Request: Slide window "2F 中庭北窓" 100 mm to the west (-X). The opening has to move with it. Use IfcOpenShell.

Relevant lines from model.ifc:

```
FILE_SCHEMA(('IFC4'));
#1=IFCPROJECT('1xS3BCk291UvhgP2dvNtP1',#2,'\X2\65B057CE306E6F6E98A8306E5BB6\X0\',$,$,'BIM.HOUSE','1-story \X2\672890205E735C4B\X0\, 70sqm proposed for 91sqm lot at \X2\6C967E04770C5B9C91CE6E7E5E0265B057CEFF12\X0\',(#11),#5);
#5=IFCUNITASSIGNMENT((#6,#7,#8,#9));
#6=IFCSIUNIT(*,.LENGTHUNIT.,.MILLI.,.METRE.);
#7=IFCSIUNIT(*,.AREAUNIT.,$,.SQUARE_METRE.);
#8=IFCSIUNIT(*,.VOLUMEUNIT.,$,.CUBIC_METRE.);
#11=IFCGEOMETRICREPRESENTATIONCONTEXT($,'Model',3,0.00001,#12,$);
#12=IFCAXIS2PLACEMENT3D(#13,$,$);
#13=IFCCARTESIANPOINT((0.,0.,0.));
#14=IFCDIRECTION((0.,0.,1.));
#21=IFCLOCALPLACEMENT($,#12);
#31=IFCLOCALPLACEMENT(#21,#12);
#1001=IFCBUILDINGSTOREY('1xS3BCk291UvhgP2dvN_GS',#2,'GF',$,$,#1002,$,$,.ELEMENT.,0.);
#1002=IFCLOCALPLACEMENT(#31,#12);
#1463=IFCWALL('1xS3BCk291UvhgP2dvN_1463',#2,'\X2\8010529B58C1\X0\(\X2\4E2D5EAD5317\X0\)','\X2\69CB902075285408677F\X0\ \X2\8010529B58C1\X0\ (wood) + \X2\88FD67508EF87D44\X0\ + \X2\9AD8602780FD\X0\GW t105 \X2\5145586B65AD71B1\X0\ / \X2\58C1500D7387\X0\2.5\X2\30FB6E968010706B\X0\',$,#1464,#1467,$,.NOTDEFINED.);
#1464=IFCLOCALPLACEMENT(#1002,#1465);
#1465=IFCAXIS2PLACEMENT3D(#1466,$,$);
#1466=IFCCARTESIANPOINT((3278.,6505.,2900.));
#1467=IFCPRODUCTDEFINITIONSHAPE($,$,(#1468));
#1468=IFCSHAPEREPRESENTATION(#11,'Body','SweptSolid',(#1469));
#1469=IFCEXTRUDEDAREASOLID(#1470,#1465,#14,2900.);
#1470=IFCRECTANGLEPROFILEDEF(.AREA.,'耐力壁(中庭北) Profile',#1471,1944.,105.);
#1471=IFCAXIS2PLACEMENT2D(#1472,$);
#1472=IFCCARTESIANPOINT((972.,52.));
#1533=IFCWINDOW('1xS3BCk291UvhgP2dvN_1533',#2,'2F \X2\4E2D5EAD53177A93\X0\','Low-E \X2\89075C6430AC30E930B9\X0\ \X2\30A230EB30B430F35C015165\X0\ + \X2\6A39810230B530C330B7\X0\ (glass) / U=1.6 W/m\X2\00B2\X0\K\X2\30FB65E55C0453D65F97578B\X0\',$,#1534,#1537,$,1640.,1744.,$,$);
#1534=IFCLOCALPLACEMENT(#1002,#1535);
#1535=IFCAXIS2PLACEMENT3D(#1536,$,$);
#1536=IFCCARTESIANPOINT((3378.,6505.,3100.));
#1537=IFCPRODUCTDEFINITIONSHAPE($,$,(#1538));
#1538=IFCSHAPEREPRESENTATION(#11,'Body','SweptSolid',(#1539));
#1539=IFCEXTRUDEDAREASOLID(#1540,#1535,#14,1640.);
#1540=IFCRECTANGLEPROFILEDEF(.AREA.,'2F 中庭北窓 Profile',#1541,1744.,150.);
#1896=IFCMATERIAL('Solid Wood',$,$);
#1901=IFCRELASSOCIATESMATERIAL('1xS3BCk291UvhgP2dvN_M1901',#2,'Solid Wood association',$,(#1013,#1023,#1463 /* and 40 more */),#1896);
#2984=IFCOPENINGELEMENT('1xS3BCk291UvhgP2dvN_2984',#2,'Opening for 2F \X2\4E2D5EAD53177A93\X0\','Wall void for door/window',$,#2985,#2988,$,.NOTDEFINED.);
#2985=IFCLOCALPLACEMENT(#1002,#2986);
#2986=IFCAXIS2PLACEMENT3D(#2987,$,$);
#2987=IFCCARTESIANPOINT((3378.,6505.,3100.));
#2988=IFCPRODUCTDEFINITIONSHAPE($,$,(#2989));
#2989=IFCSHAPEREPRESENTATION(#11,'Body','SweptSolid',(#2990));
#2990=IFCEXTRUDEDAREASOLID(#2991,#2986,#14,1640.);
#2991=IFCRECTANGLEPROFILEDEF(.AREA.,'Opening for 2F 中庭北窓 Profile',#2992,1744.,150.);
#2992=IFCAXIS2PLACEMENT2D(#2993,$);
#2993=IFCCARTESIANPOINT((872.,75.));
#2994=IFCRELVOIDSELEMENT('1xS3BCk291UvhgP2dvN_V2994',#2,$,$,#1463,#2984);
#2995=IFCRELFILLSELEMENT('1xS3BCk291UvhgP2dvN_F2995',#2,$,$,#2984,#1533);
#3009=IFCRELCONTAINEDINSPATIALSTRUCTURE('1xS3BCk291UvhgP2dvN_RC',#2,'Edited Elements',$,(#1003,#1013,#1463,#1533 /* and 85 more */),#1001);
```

```python
import ifcopenshell
import ifcopenshell.api.geometry
import ifcopenshell.util.placement

model = ifcopenshell.open("model.ifc")

window = model.by_guid("1xS3BCk291UvhgP2dvN_1533")
opening = window.FillsVoids[0].RelatingOpeningElement
wall = opening.VoidsElements[0].RelatingBuildingElement

wall_matrix = ifcopenshell.util.placement.get_local_placement(wall.ObjectPlacement)
shift = wall_matrix[:3, 0] * -100.0
before = ifcopenshell.util.placement.get_local_placement(window.ObjectPlacement)[:3, 3].copy()

# The window is not placed relative to its opening, so move both.
for product in (opening, window):
    matrix = ifcopenshell.util.placement.get_local_placement(product.ObjectPlacement)
    matrix[:3, 3] += shift
    ifcopenshell.api.geometry.edit_object_placement(model, product=product, matrix=matrix, is_si=False)

after = ifcopenshell.util.placement.get_local_placement(window.ObjectPlacement)[:3, 3]
print("window moved by", (after - before).round(3) + 0.0)

model.write("model_updated.ifc")
```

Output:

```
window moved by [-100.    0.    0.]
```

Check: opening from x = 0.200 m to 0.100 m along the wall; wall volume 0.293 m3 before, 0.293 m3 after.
